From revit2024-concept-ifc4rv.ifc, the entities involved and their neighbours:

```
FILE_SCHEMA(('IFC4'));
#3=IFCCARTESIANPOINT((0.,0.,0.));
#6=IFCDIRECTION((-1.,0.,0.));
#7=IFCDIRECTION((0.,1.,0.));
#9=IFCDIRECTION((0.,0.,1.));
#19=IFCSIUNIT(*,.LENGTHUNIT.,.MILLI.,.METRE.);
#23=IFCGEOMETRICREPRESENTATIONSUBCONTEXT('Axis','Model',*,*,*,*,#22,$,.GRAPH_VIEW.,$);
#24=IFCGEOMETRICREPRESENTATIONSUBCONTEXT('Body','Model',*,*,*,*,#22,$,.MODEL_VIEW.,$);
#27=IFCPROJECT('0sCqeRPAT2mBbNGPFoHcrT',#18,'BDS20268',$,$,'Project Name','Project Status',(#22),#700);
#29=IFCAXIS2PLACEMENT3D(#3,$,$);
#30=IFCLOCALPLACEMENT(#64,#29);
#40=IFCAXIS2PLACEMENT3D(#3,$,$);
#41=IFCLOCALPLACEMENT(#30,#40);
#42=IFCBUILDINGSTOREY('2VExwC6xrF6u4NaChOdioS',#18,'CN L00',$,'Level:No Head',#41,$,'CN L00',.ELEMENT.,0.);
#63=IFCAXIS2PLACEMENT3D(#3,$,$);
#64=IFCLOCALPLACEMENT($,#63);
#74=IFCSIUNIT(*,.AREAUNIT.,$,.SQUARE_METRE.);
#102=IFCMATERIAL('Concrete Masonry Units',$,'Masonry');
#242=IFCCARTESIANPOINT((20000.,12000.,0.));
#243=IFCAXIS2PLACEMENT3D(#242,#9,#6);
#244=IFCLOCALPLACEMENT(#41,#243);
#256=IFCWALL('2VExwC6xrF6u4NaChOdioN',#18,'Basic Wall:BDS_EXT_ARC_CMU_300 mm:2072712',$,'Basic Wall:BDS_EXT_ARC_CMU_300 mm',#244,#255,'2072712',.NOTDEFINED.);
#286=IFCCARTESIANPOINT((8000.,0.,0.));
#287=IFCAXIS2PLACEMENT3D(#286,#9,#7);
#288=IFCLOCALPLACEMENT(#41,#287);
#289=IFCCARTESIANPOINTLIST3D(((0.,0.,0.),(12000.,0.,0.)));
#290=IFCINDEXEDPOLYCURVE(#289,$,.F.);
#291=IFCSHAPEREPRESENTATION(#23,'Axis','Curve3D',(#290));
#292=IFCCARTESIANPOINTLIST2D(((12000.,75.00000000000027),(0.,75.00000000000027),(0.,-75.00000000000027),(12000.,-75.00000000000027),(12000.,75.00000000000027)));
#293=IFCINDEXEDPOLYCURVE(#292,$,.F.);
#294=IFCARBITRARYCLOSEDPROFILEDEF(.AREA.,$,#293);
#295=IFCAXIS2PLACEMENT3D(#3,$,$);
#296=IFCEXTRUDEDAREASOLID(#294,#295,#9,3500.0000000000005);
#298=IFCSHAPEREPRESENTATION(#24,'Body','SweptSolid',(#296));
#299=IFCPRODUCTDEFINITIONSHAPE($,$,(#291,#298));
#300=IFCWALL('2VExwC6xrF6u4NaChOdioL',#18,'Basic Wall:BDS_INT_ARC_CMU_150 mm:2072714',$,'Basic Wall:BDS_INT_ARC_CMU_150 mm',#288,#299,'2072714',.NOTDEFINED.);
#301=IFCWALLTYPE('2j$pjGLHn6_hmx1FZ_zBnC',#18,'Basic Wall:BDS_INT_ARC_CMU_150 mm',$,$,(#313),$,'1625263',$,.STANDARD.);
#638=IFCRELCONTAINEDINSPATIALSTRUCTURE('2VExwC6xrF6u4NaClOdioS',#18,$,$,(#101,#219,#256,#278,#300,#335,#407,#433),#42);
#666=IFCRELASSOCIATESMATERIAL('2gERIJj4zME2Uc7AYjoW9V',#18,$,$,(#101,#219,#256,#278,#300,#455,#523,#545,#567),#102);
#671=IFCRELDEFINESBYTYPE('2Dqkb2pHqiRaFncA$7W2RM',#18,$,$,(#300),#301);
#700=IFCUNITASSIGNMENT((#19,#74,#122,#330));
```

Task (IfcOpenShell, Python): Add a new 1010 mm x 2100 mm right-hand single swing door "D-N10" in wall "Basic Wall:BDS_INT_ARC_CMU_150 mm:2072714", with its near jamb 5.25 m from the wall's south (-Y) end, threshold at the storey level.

```python
import numpy as np
import ifcopenshell
import ifcopenshell.api.feature
import ifcopenshell.api.geometry
import ifcopenshell.api.root
import ifcopenshell.api.spatial
import ifcopenshell.geom
import ifcopenshell.util.element
import ifcopenshell.util.placement
import ifcopenshell.util.representation
import ifcopenshell.util.shape
import ifcopenshell.util.unit

model = ifcopenshell.open("revit2024-concept-ifc4rv.ifc")
unit_scale = ifcopenshell.util.unit.calculate_unit_scale(model)
settings = ifcopenshell.geom.settings()


def volume(element):
    """Net volume in cubic metres, openings subtracted."""
    shape = ifcopenshell.geom.create_shape(settings, element)
    return ifcopenshell.util.shape.get_volume(shape.geometry)


wall = model.by_guid("2VExwC6xrF6u4NaChOdioL")
storey = ifcopenshell.util.element.get_container(wall, ifc_class="IfcBuildingStorey")
context = ifcopenshell.util.representation.get_context(model, "Model", "Body", "MODEL_VIEW")
before = volume(wall)

width, height, from_end, sill = 1.01, 2.1, 5.25, 0.0  # metres

# The wall runs along its own X axis, and the end named is its -X end.
wall_shape = ifcopenshell.geom.create_shape(settings, wall)
x, y, z = ifcopenshell.util.shape.get_vertices(wall_shape.geometry).T
start = x.min() + from_end
face, thickness = float(y.min()), float(y.max() - y.min())
wall_matrix = ifcopenshell.util.placement.get_local_placement(wall.ObjectPlacement)
level = ifcopenshell.util.placement.get_local_placement(storey.ObjectPlacement)[2, 3]


def in_wall(x, y):
    """Placement at x, y metres in the wall's axes, at sill height."""
    matrix = wall_matrix.copy()
    matrix[:, 3] = wall_matrix @ np.array([x / unit_scale, y / unit_scale, 0.0, 1.0])
    matrix[2, 3] = level + sill / unit_scale
    return matrix


# Opening: a box that overshoots both wall faces by 50 mm.
opening = ifcopenshell.api.root.create_entity(model, ifc_class="IfcOpeningElement", predefined_type="OPENING")
box = ifcopenshell.api.geometry.add_wall_representation(
    model, context=context, length=width, height=height, thickness=thickness + 0.1
)
ifcopenshell.api.geometry.assign_representation(model, product=opening, representation=box)
ifcopenshell.api.geometry.edit_object_placement(model, product=opening, matrix=in_wall(start, face - 0.05), is_si=False)
ifcopenshell.api.feature.add_feature(model, feature=opening, element=wall)

door = ifcopenshell.api.root.create_entity(model, ifc_class="IfcDoor", name="D-N10", predefined_type="DOOR")
door.OverallWidth, door.OverallHeight = width / unit_scale, height / unit_scale
door.OperationType = "SINGLE_SWING_RIGHT"
body = ifcopenshell.api.geometry.add_door_representation(
    model,
    context=context,
    overall_width=door.OverallWidth,
    overall_height=door.OverallHeight,
    operation_type="SINGLE_SWING_RIGHT",
    lining_properties={"LiningDepth": thickness / unit_scale, "ThresholdDepth": thickness / unit_scale},
)
ifcopenshell.api.geometry.assign_representation(model, product=door, representation=body)
ifcopenshell.api.spatial.assign_container(model, products=[door], relating_structure=storey)
ifcopenshell.api.feature.add_filling(model, opening=opening, element=door)

# The lining spans the wall, so the door starts at the wall face.
ifcopenshell.api.geometry.edit_object_placement(model, product=door, matrix=in_wall(start, face), is_si=False)

after = volume(wall)

print(f"wall volume {before:.3f} -> {after:.3f} m3")

model.write("revit2024-concept-ifc4rv_rev.ifc")
```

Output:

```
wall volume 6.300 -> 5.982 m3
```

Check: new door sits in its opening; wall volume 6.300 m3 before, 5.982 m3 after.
